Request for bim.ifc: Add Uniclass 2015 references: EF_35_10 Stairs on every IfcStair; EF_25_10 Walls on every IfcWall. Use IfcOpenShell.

First a look at what the model holds.

```python
import ifcopenshell

model = ifcopenshell.open("bim.ifc")
print(model.schema)
print("classifications:", [c.Name for c in model.by_type("IfcClassification")])
for ifc_class in ("IfcDoor", "IfcRoof", "IfcStair", "IfcWall", "IfcWindow"):
    print(ifc_class, len(model.by_type(ifc_class)))
```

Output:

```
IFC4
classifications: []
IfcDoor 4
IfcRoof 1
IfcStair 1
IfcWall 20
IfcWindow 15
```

```python
import ifcopenshell
import ifcopenshell.api.classification

model = ifcopenshell.open("bim.ifc")

system = ifcopenshell.api.classification.add_classification(model, classification="Uniclass 2015")

codes = {
    "IfcStair": ("EF_35_10", "Stairs"),
    "IfcWall": ("EF_25_10", "Walls"),
}
for ifc_class, (code, name) in codes.items():
    products = model.by_type(ifc_class)
    ifcopenshell.api.classification.add_reference(
        model, products=products, classification=system, identification=code, name=name
    )
    print(code, len(products))

model.write("bim_updated.ifc")
```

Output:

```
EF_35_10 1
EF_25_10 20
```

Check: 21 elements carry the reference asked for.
